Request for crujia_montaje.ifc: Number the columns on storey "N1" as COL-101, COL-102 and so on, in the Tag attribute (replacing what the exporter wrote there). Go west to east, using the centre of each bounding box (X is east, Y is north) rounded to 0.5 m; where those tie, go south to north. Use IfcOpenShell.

First a look at what the model holds.

```python
import ifcopenshell
import ifcopenshell.util.element
import ifcopenshell.util.placement

model = ifcopenshell.open("crujia_montaje.ifc")
print(model.schema)
storey = next(s for s in model.by_type("IfcBuildingStorey") if s.Name == "N1")
columns = [e for e in ifcopenshell.util.element.get_decomposition(storey) if e.is_a("IfcColumn")]
for e in sorted(columns, key=lambda e: e.id()):
    origin = ifcopenshell.util.placement.get_local_placement(e.ObjectPlacement)[:3, 3]
    print(e.id(), e.Tag, e.Name, origin.round(2) + 0.0, sep=" | ")
```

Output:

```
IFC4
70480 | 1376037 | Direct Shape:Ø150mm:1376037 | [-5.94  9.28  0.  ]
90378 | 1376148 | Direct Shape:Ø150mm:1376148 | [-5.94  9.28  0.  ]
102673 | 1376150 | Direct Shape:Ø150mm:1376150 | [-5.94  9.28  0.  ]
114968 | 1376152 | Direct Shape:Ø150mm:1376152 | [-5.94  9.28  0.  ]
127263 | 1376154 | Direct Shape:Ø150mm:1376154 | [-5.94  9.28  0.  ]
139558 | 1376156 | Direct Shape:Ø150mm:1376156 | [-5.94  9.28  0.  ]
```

```python
import ifcopenshell
import ifcopenshell.geom
import ifcopenshell.util.element
import ifcopenshell.util.shape

model = ifcopenshell.open("crujia_montaje.ifc")
settings = ifcopenshell.geom.settings()
settings.set("use-world-coords", True)


def centre(element):
    shape = ifcopenshell.geom.create_shape(settings, element)
    return ifcopenshell.util.shape.get_bbox_centroid(shape.geometry)


storey = next(s for s in model.by_type("IfcBuildingStorey") if s.Name == "N1")
columns = [e for e in ifcopenshell.util.element.get_decomposition(storey) if e.is_a("IfcColumn")]

# Insertion points can sit at a corner or the storey origin, so sort by the geometry (in metres).
centres = {e: centre(e) for e in columns}
columns.sort(key=lambda e: (round(centres[e][0] / 0.5), centres[e][1]))

for i, e in enumerate(columns, start=1):
    number = f"COL-1{i:02d}"
    e.Tag = number
    print(e.id(), number)

model.write("crujia_montaje_edited.ifc")
```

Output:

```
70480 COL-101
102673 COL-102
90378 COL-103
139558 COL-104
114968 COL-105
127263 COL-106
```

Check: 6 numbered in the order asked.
